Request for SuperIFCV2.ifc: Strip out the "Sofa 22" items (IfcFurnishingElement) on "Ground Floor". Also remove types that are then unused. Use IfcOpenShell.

First a look at what the model holds.

```python
import ifcopenshell
import ifcopenshell.util.element

model = ifcopenshell.open("SuperIFCV2.ifc")
print(model.schema)
storey = next(s for s in model.by_type("IfcBuildingStorey") if s.Name == "Ground Floor")
furniture = [e for e in ifcopenshell.util.element.get_decomposition(storey) if e.is_a("IfcFurnishingElement")]
seen = {}
for e in furniture:
    element_type = ifcopenshell.util.element.get_type(e)
    name = element_type.Name if element_type not in (None, e) else None
    seen[name] = seen.get(name, 0) + 1
for name, count in sorted(seen.items(), key=str):
    print(count, "x", name)
```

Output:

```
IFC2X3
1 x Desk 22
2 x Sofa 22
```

```python
import ifcopenshell
import ifcopenshell.api.root
import ifcopenshell.util.element

model = ifcopenshell.open("SuperIFCV2.ifc")

storey = next(s for s in model.by_type("IfcBuildingStorey") if s.Name == "Ground Floor")
furniture = [e for e in ifcopenshell.util.element.get_decomposition(storey) if e.is_a("IfcFurnishingElement")]
targets = [e for e in furniture if (t := ifcopenshell.util.element.get_type(e)) not in (None, e) and t.Name == "Sofa 22"]
types = {ifcopenshell.util.element.get_type(e) for e in targets} - {None, *targets}

for e in targets:
    ifcopenshell.api.root.remove_product(model, product=e)
print(len(targets), "removed")

unused = [t for t in types if not ifcopenshell.util.element.get_types(t)]
for t in unused:
    ifcopenshell.api.root.remove_product(model, product=t)
print(len(unused), "unused types removed")

model.write("SuperIFCV2_rev.ifc")
```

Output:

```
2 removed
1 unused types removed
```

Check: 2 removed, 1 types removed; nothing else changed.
